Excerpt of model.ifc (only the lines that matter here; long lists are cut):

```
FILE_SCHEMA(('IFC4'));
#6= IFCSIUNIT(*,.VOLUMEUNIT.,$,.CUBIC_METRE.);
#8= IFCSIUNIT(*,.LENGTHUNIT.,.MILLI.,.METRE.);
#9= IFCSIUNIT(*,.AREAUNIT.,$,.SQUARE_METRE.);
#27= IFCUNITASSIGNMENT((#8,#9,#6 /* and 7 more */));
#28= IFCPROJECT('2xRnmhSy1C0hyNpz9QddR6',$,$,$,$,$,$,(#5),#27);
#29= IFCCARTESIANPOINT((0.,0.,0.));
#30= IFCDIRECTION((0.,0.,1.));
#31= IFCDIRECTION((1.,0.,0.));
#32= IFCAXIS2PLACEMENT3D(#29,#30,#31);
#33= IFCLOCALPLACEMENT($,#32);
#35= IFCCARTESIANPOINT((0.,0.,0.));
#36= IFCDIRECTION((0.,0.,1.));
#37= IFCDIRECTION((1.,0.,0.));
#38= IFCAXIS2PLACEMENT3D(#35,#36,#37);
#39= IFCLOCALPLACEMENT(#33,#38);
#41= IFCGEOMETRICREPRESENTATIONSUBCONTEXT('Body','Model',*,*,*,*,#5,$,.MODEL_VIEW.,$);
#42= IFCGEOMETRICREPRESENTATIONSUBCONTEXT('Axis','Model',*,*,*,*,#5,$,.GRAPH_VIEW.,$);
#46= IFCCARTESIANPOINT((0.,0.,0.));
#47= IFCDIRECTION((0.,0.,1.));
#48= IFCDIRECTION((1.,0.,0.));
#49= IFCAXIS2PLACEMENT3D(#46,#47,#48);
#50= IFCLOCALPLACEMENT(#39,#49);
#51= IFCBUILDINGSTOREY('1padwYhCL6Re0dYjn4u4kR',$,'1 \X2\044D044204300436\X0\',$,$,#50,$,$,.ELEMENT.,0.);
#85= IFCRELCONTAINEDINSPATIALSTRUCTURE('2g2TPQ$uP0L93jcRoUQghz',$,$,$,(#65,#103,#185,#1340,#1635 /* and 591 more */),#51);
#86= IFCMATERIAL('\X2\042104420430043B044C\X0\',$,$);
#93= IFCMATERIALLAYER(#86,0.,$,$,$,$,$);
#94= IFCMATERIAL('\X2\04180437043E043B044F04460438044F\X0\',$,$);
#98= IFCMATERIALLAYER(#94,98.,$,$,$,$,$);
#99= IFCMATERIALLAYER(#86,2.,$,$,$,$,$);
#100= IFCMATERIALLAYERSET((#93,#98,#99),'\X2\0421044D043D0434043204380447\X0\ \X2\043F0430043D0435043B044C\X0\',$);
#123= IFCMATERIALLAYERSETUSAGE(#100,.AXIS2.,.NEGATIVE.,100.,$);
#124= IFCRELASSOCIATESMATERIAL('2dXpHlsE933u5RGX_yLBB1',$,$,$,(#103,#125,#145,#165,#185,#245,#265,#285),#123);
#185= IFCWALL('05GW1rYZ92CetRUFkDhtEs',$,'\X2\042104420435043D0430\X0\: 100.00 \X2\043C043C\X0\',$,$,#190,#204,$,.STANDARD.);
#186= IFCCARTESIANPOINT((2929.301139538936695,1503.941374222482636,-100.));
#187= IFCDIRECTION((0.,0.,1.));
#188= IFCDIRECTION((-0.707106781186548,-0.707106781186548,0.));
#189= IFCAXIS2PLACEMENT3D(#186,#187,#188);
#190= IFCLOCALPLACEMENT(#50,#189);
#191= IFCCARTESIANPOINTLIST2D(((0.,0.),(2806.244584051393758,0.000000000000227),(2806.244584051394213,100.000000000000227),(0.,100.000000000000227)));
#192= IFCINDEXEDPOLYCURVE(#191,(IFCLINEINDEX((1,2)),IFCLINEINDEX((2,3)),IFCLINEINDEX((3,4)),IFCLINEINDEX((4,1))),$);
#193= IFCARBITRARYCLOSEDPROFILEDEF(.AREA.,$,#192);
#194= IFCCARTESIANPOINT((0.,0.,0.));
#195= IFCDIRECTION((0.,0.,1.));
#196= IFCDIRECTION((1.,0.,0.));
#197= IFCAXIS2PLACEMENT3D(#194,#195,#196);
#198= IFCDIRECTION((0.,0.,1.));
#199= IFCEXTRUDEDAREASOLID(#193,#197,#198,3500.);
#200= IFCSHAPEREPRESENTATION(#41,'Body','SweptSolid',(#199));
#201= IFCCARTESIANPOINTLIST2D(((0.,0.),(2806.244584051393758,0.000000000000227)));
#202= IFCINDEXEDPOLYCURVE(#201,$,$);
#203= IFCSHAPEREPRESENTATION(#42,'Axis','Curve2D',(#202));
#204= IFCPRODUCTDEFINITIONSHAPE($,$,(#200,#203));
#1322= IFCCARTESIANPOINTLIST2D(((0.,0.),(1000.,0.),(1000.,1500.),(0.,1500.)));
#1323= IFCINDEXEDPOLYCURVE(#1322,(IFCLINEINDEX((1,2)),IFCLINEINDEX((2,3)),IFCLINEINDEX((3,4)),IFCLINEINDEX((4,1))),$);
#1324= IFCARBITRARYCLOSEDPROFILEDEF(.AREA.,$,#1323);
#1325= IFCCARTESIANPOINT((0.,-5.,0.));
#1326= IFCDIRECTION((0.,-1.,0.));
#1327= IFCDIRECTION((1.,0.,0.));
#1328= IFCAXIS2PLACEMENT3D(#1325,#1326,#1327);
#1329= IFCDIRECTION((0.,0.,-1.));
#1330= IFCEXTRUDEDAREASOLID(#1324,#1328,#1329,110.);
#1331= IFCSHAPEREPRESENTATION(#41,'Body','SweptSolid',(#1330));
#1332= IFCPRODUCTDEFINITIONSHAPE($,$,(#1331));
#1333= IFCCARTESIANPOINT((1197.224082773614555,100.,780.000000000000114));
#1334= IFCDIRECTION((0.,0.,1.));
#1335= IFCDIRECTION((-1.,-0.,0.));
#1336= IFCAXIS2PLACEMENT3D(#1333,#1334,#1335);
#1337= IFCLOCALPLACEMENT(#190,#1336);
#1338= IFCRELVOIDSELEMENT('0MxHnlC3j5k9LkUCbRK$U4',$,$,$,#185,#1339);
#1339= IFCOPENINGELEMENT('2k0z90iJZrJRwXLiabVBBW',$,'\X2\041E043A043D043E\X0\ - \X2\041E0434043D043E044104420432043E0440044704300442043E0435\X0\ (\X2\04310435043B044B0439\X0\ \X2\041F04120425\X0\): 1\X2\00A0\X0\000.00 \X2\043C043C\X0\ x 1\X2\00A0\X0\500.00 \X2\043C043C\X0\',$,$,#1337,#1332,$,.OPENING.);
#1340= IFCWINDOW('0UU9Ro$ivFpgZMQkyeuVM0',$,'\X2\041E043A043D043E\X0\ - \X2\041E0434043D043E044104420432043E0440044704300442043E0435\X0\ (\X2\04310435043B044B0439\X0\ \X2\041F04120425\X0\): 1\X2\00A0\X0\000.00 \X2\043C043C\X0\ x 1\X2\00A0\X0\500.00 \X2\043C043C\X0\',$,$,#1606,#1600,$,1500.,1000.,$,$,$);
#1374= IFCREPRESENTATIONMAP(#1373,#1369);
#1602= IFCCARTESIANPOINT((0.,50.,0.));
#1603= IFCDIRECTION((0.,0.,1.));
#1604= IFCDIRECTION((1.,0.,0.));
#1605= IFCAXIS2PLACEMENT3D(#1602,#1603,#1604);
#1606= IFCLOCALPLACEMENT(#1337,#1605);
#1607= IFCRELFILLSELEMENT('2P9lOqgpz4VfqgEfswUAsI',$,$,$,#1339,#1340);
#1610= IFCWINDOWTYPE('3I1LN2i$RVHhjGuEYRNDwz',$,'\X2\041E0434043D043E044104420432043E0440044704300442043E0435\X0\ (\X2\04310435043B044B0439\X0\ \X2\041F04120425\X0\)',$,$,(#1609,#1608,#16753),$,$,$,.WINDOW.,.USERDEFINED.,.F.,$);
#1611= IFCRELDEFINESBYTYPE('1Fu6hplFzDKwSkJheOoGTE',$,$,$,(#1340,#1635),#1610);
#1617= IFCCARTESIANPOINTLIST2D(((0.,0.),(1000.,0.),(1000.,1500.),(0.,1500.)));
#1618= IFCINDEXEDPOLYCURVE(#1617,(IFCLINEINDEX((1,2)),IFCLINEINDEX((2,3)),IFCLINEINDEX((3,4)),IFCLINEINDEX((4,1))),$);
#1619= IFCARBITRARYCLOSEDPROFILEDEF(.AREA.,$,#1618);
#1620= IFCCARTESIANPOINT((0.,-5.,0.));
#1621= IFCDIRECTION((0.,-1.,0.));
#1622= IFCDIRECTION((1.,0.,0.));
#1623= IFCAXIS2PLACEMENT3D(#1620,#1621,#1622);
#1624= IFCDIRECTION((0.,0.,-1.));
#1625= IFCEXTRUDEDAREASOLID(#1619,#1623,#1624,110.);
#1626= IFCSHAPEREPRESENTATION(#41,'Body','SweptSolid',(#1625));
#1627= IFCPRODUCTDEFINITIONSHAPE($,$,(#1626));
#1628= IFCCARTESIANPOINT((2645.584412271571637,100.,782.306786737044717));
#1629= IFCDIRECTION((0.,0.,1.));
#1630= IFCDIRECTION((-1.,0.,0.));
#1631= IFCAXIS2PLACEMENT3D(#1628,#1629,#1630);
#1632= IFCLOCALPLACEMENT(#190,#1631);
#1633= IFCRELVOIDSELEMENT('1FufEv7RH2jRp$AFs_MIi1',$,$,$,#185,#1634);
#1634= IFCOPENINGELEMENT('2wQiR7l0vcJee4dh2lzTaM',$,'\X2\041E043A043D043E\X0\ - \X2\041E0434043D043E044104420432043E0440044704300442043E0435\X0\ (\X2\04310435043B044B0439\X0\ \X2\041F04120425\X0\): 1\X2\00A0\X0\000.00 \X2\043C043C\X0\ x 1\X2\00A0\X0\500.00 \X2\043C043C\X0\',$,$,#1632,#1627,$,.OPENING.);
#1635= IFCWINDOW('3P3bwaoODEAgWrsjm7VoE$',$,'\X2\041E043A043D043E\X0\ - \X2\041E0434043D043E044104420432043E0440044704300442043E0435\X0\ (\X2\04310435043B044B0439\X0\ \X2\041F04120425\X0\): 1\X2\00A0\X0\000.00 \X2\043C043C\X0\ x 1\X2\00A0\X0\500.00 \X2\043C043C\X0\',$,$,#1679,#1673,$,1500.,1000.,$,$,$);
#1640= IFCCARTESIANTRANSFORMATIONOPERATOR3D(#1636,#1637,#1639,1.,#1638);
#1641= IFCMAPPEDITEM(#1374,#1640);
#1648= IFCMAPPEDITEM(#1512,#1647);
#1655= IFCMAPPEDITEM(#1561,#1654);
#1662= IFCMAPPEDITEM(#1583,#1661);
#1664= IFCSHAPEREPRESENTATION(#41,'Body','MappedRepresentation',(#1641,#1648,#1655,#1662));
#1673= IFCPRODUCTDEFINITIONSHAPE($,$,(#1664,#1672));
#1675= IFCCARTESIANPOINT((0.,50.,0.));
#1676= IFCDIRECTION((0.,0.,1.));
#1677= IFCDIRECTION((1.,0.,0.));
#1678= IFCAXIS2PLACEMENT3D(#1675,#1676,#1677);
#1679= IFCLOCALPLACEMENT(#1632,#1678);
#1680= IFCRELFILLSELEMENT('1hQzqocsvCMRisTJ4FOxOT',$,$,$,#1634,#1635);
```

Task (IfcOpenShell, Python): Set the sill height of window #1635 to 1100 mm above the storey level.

```python
import numpy as np
import ifcopenshell
import ifcopenshell.api.geometry
import ifcopenshell.geom
import ifcopenshell.util.element
import ifcopenshell.util.placement
import ifcopenshell.util.shape
import ifcopenshell.util.unit

model = ifcopenshell.open("model.ifc")
unit_scale = ifcopenshell.util.unit.calculate_unit_scale(model)

window = model.by_id(1635)
opening = window.FillsVoids[0].RelatingOpeningElement
storey = ifcopenshell.util.element.get_container(window, ifc_class="IfcBuildingStorey")
level = ifcopenshell.util.placement.get_local_placement(storey.ObjectPlacement)[2, 3]

# The opening's origin need not be at the sill, so measure its lowest point.
shape = ifcopenshell.geom.create_shape(ifcopenshell.geom.settings(), opening)
bottom = ifcopenshell.util.shape.get_shape_bottom_elevation(shape, shape.geometry) / unit_scale
dz = level + 1100.0 - bottom

shift = np.array([0.0, 0.0, dz])
# The window is placed relative to its opening, so it follows when the opening moves.
matrix = ifcopenshell.util.placement.get_local_placement(opening.ObjectPlacement)
matrix[:3, 3] += shift
ifcopenshell.api.geometry.edit_object_placement(
    model, product=opening, matrix=matrix, is_si=False, should_transform_children=True
)

print(f"moved by {dz * unit_scale:+.3f} m")

model.write("model-out.ifc")
```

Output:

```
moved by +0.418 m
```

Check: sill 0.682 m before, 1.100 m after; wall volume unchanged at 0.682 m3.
